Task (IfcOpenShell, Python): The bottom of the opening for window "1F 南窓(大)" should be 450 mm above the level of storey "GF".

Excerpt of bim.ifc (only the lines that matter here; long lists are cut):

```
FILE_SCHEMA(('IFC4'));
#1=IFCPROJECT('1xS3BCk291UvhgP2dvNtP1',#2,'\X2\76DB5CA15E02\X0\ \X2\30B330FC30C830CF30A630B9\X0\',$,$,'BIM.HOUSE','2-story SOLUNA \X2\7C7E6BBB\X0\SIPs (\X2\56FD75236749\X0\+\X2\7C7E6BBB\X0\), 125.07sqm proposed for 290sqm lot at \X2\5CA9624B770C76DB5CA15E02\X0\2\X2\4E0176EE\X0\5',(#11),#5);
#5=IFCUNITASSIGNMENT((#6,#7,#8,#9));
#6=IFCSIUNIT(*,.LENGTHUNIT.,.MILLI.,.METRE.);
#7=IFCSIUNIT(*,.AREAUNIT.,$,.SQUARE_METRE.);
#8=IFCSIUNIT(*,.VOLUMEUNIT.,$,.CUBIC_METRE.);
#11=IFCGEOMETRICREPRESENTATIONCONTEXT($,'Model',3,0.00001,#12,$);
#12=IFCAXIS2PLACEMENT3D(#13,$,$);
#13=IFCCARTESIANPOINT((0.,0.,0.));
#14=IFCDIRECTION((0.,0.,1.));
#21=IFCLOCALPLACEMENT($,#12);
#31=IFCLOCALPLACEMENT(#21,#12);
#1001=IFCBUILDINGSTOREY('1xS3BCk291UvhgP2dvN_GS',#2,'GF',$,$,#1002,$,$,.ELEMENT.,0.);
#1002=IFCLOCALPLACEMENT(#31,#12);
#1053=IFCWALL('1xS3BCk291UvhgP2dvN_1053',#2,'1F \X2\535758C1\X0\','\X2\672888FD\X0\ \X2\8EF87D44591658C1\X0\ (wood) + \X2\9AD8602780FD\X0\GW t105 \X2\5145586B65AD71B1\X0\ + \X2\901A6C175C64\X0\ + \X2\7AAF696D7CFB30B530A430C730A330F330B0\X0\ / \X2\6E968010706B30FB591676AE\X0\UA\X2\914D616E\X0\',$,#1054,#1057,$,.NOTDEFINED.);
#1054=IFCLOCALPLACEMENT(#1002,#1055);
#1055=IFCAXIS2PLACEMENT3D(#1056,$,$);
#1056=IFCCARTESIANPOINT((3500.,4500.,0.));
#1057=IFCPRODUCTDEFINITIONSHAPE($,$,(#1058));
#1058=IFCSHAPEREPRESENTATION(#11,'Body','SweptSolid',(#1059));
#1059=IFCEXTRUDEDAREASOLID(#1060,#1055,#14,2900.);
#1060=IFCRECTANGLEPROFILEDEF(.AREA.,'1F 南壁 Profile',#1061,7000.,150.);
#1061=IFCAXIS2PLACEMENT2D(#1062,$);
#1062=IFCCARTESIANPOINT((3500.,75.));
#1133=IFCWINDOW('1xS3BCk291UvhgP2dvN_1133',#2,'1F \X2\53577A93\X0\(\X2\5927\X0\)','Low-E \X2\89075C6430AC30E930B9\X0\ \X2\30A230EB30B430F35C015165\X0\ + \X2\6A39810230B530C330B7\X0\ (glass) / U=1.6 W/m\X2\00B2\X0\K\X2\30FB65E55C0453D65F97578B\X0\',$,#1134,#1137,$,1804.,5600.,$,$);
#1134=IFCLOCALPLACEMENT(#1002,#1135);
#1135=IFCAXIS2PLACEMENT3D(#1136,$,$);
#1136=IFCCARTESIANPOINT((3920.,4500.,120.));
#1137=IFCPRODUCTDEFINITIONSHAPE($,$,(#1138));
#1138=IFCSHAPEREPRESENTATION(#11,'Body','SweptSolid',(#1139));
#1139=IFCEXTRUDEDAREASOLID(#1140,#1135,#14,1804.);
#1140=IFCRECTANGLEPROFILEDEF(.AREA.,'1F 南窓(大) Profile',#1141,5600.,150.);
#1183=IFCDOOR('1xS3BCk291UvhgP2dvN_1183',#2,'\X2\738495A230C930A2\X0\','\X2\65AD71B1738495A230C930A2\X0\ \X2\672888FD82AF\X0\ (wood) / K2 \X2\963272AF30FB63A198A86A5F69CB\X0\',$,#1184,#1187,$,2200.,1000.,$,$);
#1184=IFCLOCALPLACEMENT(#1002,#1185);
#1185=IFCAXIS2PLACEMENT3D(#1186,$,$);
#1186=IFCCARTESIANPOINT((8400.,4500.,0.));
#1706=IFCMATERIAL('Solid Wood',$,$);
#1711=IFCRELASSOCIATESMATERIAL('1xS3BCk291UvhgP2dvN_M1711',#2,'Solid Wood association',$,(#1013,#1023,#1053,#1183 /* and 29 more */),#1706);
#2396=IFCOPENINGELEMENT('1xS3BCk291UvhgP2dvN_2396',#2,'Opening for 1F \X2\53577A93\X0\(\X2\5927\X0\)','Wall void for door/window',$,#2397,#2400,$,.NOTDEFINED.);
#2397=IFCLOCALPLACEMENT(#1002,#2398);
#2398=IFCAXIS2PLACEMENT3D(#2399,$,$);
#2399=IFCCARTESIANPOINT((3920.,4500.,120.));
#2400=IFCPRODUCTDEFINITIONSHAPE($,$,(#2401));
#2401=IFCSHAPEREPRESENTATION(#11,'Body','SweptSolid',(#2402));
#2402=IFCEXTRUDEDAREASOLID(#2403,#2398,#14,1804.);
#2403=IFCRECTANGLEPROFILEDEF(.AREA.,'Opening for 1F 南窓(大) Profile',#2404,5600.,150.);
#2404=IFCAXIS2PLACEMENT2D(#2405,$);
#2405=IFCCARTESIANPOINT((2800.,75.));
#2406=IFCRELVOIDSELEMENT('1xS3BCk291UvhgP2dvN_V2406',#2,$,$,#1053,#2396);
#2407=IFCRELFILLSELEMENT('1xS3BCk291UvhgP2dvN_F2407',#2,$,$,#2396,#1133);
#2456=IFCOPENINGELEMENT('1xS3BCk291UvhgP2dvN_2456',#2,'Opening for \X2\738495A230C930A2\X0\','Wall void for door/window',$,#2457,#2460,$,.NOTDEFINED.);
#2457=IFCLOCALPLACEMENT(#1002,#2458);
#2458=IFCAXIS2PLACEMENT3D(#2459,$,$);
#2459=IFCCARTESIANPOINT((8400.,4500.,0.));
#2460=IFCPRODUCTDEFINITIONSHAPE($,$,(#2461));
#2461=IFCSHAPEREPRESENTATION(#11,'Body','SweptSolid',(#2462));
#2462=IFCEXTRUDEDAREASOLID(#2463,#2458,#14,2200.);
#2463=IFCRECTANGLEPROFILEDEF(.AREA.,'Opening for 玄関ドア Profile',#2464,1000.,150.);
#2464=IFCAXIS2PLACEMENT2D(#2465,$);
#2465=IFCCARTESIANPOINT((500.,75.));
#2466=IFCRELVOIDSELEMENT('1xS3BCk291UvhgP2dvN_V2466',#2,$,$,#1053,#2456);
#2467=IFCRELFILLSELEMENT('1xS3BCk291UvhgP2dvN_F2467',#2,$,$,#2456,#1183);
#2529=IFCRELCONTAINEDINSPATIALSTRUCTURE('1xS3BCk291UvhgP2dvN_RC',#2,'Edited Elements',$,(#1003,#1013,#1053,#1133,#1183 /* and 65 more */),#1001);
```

```python
import numpy as np
import ifcopenshell
import ifcopenshell.api.geometry
import ifcopenshell.geom
import ifcopenshell.util.element
import ifcopenshell.util.placement
import ifcopenshell.util.shape
import ifcopenshell.util.unit

model = ifcopenshell.open("bim.ifc")
unit_scale = ifcopenshell.util.unit.calculate_unit_scale(model)

window = model.by_guid("1xS3BCk291UvhgP2dvN_1133")
opening = window.FillsVoids[0].RelatingOpeningElement
storey = ifcopenshell.util.element.get_container(window, ifc_class="IfcBuildingStorey")
level = ifcopenshell.util.placement.get_local_placement(storey.ObjectPlacement)[2, 3]

# The opening's origin need not be at the sill, so measure its lowest point.
shape = ifcopenshell.geom.create_shape(ifcopenshell.geom.settings(), opening)
bottom = ifcopenshell.util.shape.get_shape_bottom_elevation(shape, shape.geometry) / unit_scale
dz = level + 0.45 / unit_scale - bottom

shift = np.array([0.0, 0.0, dz])
# The window is not placed relative to its opening, so move both.
for product in (opening, window):
    matrix = ifcopenshell.util.placement.get_local_placement(product.ObjectPlacement)
    matrix[:3, 3] += shift
    ifcopenshell.api.geometry.edit_object_placement(model, product=product, matrix=matrix, is_si=False)

print(f"moved by {dz * unit_scale:+.3f} m")

model.write("bim_edited.ifc")
```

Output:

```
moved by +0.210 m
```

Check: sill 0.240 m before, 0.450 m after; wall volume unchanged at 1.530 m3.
